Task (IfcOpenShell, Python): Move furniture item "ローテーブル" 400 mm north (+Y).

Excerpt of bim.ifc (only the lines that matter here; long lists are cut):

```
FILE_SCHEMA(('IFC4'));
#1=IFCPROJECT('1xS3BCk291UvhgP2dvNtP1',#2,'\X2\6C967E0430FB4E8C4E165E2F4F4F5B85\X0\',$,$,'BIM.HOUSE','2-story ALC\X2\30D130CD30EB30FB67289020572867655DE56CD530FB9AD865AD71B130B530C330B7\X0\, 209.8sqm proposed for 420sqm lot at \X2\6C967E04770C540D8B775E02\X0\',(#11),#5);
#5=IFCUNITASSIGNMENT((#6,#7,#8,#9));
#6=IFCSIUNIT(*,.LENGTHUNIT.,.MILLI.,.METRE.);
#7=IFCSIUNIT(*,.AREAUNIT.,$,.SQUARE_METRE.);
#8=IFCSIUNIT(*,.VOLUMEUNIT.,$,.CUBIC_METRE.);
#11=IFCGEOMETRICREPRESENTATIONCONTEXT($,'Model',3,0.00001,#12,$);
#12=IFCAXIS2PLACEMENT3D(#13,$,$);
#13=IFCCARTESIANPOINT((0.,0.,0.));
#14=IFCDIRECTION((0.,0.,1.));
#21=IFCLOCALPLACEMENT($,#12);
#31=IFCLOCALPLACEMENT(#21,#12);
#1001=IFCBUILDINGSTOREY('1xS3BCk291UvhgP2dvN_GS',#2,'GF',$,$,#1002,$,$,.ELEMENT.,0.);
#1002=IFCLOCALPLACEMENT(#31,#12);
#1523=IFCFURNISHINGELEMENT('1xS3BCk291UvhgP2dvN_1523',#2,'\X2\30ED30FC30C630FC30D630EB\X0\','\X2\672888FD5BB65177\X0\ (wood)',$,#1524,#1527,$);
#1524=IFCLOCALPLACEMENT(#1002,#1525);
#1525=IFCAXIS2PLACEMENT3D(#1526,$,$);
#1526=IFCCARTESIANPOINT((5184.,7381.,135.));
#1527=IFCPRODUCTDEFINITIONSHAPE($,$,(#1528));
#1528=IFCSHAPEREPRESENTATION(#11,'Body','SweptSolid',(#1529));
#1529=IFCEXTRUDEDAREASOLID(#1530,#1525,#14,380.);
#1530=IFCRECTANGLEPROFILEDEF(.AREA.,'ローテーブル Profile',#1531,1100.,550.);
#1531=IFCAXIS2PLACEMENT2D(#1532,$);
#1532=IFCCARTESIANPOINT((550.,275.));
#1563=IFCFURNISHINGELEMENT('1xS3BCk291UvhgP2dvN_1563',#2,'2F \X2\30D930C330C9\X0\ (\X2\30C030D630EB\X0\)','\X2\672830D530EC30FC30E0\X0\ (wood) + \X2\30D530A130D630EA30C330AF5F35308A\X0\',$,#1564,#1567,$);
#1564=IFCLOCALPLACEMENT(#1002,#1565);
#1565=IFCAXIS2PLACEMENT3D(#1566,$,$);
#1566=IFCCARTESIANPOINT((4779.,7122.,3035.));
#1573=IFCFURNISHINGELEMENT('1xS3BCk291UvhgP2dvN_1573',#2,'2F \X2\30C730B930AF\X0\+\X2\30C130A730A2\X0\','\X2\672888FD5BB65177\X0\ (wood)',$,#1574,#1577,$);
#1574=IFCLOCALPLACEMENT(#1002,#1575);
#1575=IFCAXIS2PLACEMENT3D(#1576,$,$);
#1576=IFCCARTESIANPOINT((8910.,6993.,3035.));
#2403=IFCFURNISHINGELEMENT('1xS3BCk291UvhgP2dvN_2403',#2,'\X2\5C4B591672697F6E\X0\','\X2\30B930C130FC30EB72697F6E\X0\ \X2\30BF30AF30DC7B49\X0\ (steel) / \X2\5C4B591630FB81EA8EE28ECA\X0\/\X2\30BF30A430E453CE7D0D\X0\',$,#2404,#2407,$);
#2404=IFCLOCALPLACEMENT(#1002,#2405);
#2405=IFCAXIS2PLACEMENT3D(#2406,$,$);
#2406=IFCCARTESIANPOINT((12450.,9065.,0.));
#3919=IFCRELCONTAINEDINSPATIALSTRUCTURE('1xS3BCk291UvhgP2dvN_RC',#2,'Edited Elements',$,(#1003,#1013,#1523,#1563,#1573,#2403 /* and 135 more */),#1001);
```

```python
import ifcopenshell
import ifcopenshell.api.geometry
import ifcopenshell.util.placement
import ifcopenshell.util.unit

model = ifcopenshell.open("bim.ifc")
unit_scale = ifcopenshell.util.unit.calculate_unit_scale(model)

item = model.by_id(1523)
matrix = ifcopenshell.util.placement.get_local_placement(item.ObjectPlacement)
matrix[1, 3] += 0.4 / unit_scale
ifcopenshell.api.geometry.edit_object_placement(model, product=item, matrix=matrix, is_si=False)

print(ifcopenshell.util.placement.get_local_placement(item.ObjectPlacement).round(3) + 0.0)

model.write("bim_edited.ifc")
```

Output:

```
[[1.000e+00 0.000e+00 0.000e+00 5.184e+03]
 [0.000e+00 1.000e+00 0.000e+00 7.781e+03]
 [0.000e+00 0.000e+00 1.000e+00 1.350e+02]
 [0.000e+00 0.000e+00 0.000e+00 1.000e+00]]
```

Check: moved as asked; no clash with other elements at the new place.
